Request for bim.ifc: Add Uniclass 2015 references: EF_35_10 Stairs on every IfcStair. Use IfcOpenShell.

First a look at what the model holds.

```python
import ifcopenshell

model = ifcopenshell.open("bim.ifc")
print(model.schema)
print("classifications:", [c.Name for c in model.by_type("IfcClassification")])
for ifc_class in ("IfcDoor", "IfcRoof", "IfcStair", "IfcWall", "IfcWindow"):
    print(ifc_class, len(model.by_type(ifc_class)))
```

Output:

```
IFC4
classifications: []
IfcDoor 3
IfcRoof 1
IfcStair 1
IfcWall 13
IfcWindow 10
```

```python
import ifcopenshell
import ifcopenshell.api.classification

model = ifcopenshell.open("bim.ifc")

system = ifcopenshell.api.classification.add_classification(model, classification="Uniclass 2015")

codes = {
    "IfcStair": ("EF_35_10", "Stairs"),
}
for ifc_class, (code, name) in codes.items():
    products = model.by_type(ifc_class)
    ifcopenshell.api.classification.add_reference(
        model, products=products, classification=system, identification=code, name=name
    )
    print(code, len(products))

model.write("bim_edited.ifc")
```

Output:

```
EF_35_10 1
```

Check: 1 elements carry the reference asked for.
